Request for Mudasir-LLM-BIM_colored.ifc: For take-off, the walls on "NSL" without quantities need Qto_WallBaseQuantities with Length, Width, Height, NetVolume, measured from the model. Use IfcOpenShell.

First a look at what the model holds.

```python
import ifcopenshell
import ifcopenshell.util.element
import ifcopenshell.util.unit

model = ifcopenshell.open("Mudasir-LLM-BIM_colored.ifc")
print(model.schema)
for unit_type in ("LENGTHUNIT", "AREAUNIT", "VOLUMEUNIT"):
    print(unit_type, ifcopenshell.util.unit.calculate_unit_scale(model, unit_type))
storey = next(s for s in model.by_type("IfcBuildingStorey") if s.Name == "NSL")
walls = [e for e in ifcopenshell.util.element.get_decomposition(storey) if e.is_a("IfcWall")]
for e in sorted(walls, key=lambda e: e.id()):
    print(e.id(), e.is_a(), e.Name, list(ifcopenshell.util.element.get_psets(e, qtos_only=True)), sep=" | ")
```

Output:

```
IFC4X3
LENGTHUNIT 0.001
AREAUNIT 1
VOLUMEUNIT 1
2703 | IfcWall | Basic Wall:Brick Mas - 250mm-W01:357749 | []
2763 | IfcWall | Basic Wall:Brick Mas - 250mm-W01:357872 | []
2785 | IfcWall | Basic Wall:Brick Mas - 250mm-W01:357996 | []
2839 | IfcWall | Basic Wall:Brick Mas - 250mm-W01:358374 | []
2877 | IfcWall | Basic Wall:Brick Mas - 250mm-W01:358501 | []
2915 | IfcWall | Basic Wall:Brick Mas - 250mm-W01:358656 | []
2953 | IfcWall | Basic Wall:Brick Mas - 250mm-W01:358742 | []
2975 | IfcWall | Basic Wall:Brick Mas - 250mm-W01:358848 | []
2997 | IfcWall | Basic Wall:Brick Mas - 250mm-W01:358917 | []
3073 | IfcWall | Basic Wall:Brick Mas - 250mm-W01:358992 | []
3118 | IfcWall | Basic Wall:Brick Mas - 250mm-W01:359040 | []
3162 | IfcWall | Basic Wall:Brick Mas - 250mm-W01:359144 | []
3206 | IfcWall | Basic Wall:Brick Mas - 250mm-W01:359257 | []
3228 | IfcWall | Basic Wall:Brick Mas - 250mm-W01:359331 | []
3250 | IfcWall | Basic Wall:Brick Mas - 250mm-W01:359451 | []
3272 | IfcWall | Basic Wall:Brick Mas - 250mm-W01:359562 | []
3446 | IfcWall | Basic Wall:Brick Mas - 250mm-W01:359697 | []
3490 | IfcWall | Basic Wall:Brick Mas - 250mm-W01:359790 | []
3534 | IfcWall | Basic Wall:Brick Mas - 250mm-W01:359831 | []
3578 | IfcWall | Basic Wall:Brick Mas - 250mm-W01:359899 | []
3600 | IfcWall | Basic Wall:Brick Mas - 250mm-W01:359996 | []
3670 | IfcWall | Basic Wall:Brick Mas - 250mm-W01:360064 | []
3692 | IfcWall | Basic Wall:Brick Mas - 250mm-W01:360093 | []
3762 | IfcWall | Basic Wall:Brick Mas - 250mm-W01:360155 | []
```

```python
import ifcopenshell
import ifcopenshell.api.pset
import ifcopenshell.geom
import ifcopenshell.util.element
import ifcopenshell.util.shape
import ifcopenshell.util.unit

model = ifcopenshell.open("Mudasir-LLM-BIM_colored.ifc")
unit_scale = ifcopenshell.util.unit.calculate_unit_scale(model)
volume_scale = ifcopenshell.util.unit.calculate_unit_scale(model, "VOLUMEUNIT")
settings = ifcopenshell.geom.settings()

storey = next(s for s in model.by_type("IfcBuildingStorey") if s.Name == "NSL")
walls = [e for e in ifcopenshell.util.element.get_decomposition(storey) if e.is_a("IfcWall")]

for e in sorted(walls, key=lambda e: e.id()):
    if ifcopenshell.util.element.get_psets(e, qtos_only=True, should_inherit=False):
        continue
    # Geometry comes back in metres, in the element's own axes.
    shape = ifcopenshell.geom.create_shape(settings, e)
    values = {
        "Length": ifcopenshell.util.shape.get_x(shape.geometry) / unit_scale,
        "Width": ifcopenshell.util.shape.get_y(shape.geometry) / unit_scale,
        "Height": ifcopenshell.util.shape.get_z(shape.geometry) / unit_scale,
        "NetVolume": ifcopenshell.util.shape.get_volume(shape.geometry) / volume_scale,
    }
    qto = ifcopenshell.api.pset.add_qto(model, product=e, name="Qto_WallBaseQuantities")
    ifcopenshell.api.pset.edit_qto(model, qto=qto, properties=values)
    print(e.id(), {k: round(v, 3) for k, v in values.items()})

model.write("Mudasir-LLM-BIM_colored_updated.ifc")
```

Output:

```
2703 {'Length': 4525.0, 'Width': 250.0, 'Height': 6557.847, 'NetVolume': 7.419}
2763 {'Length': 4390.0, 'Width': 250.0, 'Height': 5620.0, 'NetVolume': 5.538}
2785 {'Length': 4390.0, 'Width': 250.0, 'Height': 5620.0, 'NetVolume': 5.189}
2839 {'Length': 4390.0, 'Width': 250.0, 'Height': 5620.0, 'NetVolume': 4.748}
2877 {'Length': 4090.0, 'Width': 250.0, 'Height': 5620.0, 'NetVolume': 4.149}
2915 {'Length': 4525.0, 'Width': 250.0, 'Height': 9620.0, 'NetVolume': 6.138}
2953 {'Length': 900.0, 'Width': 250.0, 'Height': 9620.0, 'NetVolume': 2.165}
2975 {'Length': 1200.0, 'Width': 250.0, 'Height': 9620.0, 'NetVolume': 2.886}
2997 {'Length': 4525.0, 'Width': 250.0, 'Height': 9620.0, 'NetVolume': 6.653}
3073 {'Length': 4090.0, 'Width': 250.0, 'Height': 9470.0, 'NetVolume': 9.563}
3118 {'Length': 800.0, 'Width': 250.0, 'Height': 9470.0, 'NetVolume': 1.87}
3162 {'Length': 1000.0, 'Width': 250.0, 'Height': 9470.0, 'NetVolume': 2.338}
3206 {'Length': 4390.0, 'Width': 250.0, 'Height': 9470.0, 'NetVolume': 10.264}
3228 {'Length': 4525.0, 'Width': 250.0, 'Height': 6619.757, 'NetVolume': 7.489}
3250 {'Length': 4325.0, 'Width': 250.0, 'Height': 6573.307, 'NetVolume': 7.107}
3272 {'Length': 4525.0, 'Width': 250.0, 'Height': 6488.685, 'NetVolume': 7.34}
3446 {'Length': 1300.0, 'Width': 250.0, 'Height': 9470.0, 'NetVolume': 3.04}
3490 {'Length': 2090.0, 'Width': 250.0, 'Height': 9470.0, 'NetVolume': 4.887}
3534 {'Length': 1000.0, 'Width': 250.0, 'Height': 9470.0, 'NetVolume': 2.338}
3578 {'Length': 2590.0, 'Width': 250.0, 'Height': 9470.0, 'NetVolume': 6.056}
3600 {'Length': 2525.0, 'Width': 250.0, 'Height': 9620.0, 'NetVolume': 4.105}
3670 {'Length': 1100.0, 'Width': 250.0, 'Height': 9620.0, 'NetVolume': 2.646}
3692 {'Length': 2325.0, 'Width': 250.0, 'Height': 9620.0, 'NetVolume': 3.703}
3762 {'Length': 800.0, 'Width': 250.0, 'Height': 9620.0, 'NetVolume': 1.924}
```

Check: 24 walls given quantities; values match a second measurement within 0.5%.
